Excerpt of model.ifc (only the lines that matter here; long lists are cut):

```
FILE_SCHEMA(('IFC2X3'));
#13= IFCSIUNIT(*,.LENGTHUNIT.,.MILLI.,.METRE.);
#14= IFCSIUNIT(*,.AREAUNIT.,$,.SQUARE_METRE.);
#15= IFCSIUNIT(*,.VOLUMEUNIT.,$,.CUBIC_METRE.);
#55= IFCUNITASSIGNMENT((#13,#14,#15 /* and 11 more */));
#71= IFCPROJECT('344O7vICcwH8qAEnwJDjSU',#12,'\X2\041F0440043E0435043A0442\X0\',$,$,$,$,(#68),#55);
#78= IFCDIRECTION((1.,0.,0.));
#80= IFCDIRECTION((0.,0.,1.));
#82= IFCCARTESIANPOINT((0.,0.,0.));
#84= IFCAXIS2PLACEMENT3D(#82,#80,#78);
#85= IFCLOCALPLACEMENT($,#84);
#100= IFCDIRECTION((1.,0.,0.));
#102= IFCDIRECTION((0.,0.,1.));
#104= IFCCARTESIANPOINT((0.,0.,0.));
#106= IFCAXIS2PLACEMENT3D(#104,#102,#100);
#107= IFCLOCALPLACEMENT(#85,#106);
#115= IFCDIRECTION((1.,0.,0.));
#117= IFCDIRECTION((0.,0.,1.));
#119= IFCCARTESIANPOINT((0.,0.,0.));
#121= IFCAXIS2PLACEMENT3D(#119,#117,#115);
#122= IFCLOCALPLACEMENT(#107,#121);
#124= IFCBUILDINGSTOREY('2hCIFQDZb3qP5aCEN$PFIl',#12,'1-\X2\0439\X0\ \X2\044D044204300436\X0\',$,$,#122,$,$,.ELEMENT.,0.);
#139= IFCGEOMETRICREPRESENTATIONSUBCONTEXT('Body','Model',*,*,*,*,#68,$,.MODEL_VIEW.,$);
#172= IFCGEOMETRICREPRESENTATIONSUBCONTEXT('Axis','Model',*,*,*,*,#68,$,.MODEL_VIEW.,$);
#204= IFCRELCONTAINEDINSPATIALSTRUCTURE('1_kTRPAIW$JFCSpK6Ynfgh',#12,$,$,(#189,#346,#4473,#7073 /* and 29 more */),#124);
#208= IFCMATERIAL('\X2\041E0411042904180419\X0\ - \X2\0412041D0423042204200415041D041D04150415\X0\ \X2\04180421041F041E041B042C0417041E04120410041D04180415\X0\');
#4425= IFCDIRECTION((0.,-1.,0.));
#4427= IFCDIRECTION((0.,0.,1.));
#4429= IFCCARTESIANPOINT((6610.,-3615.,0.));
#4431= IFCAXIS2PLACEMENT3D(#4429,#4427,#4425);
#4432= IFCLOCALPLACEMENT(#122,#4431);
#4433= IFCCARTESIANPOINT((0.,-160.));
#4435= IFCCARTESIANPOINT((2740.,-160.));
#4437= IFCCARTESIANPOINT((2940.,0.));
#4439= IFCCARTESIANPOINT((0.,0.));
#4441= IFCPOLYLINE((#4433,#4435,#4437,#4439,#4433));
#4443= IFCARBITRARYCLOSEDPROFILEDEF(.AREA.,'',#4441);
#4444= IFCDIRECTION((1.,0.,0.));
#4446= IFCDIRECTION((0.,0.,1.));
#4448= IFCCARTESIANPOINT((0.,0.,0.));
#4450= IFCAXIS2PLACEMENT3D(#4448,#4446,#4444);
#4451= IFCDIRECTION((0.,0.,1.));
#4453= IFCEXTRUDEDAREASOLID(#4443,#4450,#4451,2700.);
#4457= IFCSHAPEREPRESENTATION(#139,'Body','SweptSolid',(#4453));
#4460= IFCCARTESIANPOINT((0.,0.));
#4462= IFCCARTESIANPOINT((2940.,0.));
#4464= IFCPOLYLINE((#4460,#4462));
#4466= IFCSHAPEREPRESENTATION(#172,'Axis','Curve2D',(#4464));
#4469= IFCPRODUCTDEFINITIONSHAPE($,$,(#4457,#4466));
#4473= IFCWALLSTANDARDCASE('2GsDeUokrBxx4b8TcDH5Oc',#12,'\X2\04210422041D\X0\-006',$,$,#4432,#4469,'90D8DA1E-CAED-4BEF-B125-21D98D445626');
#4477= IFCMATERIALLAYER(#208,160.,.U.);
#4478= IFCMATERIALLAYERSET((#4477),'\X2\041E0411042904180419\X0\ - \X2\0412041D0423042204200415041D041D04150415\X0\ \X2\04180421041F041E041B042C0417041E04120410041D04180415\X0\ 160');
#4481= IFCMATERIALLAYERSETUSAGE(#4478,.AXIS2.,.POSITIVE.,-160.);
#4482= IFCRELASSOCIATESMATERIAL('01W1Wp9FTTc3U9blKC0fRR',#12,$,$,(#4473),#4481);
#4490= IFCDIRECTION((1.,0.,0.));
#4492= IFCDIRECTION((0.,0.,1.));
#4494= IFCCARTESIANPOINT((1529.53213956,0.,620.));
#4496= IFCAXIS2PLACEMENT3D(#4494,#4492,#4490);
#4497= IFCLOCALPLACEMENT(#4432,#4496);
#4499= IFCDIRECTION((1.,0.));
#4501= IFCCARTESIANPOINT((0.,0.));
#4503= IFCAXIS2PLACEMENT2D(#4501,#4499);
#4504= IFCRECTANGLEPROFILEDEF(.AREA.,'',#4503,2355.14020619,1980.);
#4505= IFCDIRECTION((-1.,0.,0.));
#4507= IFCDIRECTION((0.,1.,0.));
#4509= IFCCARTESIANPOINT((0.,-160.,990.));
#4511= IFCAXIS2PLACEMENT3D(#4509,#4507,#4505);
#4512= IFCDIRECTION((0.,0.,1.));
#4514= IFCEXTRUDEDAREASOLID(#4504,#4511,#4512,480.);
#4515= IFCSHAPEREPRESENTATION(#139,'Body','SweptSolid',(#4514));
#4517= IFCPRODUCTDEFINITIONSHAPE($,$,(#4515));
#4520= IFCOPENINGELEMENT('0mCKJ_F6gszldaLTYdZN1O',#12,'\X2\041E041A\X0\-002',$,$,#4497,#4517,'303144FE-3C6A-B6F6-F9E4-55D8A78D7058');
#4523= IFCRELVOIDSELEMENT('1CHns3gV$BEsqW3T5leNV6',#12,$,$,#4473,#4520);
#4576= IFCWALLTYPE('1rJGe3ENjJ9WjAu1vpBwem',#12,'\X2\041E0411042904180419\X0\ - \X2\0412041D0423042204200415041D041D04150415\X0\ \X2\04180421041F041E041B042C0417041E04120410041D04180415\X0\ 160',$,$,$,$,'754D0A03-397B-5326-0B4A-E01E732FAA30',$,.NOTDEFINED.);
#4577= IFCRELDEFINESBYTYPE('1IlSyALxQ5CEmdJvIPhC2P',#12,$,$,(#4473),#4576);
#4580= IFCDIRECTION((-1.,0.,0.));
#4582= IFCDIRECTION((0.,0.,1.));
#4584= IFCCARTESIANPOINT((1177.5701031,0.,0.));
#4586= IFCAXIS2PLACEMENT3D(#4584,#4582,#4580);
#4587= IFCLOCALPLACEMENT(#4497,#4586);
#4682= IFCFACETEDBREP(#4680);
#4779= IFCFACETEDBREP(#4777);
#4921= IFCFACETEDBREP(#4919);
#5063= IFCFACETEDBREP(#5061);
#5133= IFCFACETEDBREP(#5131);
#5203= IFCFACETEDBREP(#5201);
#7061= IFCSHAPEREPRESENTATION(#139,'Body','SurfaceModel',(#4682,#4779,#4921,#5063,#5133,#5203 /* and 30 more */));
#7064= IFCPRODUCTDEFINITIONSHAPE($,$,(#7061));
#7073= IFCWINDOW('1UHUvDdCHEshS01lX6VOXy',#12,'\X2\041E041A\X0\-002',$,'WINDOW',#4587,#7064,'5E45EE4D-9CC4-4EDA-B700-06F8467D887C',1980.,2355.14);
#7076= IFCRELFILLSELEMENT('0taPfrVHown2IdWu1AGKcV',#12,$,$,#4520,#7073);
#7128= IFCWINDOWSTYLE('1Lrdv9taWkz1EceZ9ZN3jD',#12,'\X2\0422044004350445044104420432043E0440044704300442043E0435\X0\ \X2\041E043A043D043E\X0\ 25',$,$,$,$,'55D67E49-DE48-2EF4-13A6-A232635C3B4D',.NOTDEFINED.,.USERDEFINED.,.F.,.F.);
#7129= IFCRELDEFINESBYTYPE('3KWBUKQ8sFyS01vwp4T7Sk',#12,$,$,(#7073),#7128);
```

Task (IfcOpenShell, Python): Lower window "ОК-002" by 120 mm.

```python
import numpy as np
import ifcopenshell
import ifcopenshell.api.geometry
import ifcopenshell.util.placement
import ifcopenshell.util.unit

model = ifcopenshell.open("model.ifc")
unit_scale = ifcopenshell.util.unit.calculate_unit_scale(model)

window = model.by_id(7073)
opening = window.FillsVoids[0].RelatingOpeningElement
dz = -0.12 / unit_scale

shift = np.array([0.0, 0.0, dz])
# The window is placed relative to its opening, so it follows when the opening moves.
matrix = ifcopenshell.util.placement.get_local_placement(opening.ObjectPlacement)
matrix[:3, 3] += shift
ifcopenshell.api.geometry.edit_object_placement(
    model, product=opening, matrix=matrix, is_si=False, should_transform_children=True
)

print(f"moved by {dz * unit_scale:+.3f} m")

model.write("model_updated.ifc")
```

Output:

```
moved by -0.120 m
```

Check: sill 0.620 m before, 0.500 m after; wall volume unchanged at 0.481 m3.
